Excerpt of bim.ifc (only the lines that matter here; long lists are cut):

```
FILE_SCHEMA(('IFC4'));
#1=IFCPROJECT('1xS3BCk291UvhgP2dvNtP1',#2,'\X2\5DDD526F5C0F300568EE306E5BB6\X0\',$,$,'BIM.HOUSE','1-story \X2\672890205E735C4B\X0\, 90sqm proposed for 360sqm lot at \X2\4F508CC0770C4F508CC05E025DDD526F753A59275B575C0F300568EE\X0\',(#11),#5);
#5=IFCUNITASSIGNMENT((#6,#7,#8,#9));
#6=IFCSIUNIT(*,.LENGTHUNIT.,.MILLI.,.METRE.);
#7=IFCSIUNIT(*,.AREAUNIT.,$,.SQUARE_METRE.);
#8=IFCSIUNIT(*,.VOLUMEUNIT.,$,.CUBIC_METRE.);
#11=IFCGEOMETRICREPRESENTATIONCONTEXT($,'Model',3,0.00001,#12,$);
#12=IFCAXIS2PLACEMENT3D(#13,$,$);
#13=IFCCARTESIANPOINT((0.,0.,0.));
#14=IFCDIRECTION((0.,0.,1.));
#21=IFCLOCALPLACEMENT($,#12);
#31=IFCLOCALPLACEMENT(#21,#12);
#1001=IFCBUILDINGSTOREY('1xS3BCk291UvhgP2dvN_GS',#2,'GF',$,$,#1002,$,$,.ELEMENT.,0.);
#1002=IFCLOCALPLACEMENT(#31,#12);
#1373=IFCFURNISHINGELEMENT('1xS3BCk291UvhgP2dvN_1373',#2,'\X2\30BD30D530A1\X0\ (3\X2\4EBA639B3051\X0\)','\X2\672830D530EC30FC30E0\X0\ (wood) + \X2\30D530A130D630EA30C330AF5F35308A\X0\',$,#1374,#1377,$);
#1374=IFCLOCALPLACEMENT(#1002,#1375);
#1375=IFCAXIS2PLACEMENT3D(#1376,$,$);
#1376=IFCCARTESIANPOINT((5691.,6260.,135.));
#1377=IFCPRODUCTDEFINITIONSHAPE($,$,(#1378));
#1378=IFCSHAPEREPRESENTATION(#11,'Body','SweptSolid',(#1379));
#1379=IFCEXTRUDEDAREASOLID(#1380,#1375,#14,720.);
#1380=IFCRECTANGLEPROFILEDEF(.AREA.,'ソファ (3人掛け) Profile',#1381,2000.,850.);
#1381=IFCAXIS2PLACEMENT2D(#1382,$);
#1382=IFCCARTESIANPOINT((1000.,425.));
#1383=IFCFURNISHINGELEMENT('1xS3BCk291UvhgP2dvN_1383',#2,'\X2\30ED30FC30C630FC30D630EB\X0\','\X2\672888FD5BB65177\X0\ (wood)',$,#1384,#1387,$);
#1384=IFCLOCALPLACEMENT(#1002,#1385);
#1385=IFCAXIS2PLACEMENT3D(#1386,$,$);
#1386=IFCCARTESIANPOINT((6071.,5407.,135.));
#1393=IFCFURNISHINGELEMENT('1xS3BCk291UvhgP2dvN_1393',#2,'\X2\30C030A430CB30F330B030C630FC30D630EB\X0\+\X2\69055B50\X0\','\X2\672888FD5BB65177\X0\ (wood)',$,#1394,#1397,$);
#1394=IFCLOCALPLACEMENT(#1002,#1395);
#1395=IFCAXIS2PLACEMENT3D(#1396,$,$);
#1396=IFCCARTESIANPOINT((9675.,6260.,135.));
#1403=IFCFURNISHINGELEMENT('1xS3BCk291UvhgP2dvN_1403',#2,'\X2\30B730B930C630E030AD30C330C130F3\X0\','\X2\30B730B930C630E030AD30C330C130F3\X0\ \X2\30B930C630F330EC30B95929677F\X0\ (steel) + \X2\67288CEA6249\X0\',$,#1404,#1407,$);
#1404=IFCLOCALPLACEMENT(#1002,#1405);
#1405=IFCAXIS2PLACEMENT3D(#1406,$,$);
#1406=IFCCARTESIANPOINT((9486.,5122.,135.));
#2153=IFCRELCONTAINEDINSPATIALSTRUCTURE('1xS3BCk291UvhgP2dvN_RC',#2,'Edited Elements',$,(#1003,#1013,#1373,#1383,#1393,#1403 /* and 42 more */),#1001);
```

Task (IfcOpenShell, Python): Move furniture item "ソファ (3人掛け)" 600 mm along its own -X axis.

```python
import ifcopenshell
import ifcopenshell.api.geometry
import ifcopenshell.util.placement

model = ifcopenshell.open("bim.ifc")

item = model.by_guid("1xS3BCk291UvhgP2dvN_1373")
matrix = ifcopenshell.util.placement.get_local_placement(item.ObjectPlacement)
matrix[:3, 3] -= matrix[:3, 0] * 600.0
ifcopenshell.api.geometry.edit_object_placement(model, product=item, matrix=matrix, is_si=False)

print(ifcopenshell.util.placement.get_local_placement(item.ObjectPlacement).round(3) + 0.0)

model.write("bim_updated.ifc")
```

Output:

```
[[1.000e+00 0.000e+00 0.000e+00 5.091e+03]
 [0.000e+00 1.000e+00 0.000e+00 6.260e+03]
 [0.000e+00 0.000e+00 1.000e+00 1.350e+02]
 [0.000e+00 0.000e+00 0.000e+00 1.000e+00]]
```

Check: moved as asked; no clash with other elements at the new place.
